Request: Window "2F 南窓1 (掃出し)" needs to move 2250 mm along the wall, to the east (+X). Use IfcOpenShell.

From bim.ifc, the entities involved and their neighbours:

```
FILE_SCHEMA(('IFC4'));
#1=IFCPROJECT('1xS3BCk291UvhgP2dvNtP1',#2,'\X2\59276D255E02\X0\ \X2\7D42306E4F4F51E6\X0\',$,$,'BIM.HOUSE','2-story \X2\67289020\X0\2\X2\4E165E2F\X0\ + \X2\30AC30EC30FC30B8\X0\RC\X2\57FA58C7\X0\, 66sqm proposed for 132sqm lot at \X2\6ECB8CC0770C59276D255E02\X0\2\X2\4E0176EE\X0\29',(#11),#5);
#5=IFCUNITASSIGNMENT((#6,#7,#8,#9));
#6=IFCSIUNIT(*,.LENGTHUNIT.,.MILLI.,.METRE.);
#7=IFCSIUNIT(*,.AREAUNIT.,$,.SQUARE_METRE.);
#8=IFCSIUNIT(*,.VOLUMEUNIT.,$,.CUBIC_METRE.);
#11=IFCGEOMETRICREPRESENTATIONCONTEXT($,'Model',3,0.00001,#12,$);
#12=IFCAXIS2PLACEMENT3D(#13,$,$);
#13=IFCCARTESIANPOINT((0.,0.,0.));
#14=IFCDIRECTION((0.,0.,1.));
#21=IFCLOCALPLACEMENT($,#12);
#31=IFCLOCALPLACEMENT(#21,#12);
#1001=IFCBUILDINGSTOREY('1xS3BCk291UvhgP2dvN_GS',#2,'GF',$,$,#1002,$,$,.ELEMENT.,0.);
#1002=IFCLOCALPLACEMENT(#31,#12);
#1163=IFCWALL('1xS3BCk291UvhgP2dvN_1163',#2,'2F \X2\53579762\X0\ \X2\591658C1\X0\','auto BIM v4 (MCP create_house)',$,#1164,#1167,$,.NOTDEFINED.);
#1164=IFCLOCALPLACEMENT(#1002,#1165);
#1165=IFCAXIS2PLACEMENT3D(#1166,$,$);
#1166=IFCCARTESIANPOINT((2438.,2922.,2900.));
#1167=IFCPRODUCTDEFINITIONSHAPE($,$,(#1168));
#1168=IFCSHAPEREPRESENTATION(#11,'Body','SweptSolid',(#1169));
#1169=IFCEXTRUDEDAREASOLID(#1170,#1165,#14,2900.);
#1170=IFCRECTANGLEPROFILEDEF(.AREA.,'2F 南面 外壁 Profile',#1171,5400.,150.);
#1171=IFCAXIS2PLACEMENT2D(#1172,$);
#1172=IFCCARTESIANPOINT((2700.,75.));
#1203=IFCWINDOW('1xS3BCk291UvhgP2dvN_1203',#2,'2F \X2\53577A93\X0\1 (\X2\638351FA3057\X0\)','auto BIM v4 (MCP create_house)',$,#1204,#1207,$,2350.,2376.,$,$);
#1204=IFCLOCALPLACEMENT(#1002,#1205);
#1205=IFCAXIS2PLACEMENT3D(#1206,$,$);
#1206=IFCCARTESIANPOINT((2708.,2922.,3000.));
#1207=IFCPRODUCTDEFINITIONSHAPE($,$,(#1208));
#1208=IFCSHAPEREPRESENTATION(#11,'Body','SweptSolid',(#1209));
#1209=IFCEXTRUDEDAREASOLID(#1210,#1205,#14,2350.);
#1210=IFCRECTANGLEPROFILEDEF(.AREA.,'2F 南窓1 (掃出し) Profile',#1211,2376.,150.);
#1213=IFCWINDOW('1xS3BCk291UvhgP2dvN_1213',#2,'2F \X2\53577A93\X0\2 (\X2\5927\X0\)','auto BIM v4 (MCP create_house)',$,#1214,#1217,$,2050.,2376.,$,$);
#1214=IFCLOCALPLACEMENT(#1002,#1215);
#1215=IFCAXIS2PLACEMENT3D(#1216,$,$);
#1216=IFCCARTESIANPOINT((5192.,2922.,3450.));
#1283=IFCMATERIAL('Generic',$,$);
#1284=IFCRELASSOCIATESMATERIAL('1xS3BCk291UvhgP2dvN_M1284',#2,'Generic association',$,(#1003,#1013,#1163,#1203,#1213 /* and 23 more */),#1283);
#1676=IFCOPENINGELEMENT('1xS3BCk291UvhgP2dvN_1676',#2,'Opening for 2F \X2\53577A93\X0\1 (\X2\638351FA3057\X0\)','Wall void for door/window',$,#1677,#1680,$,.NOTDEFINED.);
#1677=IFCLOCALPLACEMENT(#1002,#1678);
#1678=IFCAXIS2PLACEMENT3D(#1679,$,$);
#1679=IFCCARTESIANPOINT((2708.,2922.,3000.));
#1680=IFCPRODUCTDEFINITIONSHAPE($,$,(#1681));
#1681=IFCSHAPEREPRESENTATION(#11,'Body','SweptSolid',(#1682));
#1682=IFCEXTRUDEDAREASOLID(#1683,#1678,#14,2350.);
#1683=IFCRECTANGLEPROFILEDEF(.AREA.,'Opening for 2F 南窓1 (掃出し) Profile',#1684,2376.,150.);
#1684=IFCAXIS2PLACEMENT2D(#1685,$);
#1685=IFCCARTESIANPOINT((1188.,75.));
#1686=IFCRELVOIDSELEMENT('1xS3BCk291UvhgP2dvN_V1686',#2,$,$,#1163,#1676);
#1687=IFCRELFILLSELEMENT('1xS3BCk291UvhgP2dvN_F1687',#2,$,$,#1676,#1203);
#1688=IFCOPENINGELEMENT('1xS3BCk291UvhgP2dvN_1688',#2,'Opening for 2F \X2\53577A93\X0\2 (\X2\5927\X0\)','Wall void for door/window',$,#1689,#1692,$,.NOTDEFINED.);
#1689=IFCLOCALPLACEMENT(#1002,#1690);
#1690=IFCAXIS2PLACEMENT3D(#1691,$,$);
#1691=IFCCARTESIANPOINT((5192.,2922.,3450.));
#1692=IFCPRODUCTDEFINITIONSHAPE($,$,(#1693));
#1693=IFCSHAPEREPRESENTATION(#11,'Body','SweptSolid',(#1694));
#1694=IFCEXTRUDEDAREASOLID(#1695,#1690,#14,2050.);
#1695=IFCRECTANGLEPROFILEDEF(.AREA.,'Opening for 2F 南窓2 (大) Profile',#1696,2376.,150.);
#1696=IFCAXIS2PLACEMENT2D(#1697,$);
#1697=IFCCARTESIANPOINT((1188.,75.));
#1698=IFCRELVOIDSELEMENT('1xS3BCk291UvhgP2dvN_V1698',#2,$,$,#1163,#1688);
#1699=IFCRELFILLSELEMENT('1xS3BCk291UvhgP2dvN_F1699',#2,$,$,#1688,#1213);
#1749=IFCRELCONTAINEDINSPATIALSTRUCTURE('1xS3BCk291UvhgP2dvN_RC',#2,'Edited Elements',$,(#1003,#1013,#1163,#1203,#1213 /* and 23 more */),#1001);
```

```python
import ifcopenshell
import ifcopenshell.api.geometry
import ifcopenshell.util.placement
import ifcopenshell.util.unit

model = ifcopenshell.open("bim.ifc")
unit_scale = ifcopenshell.util.unit.calculate_unit_scale(model)

window = model.by_guid("1xS3BCk291UvhgP2dvN_1203")
opening = window.FillsVoids[0].RelatingOpeningElement
wall = opening.VoidsElements[0].RelatingBuildingElement

wall_matrix = ifcopenshell.util.placement.get_local_placement(wall.ObjectPlacement)
shift = wall_matrix[:3, 0] * 2.25 / unit_scale
before = ifcopenshell.util.placement.get_local_placement(window.ObjectPlacement)[:3, 3].copy()

# The window is not placed relative to its opening, so move both.
for product in (opening, window):
    matrix = ifcopenshell.util.placement.get_local_placement(product.ObjectPlacement)
    matrix[:3, 3] += shift
    ifcopenshell.api.geometry.edit_object_placement(model, product=product, matrix=matrix, is_si=False)

after = ifcopenshell.util.placement.get_local_placement(window.ObjectPlacement)[:3, 3]
print("window moved by", (after - before).round(3) + 0.0)

model.write("bim_updated.ifc")
```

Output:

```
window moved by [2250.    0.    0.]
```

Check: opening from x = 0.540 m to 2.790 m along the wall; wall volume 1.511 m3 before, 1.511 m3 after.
